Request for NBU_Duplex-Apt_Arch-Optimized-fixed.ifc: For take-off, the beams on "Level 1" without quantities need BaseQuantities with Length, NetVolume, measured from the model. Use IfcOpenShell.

First a look at what the model holds.

```python
import ifcopenshell
import ifcopenshell.util.element
import ifcopenshell.util.unit

model = ifcopenshell.open("NBU_Duplex-Apt_Arch-Optimized-fixed.ifc")
print(model.schema)
for unit_type in ("LENGTHUNIT", "AREAUNIT", "VOLUMEUNIT"):
    print(unit_type, ifcopenshell.util.unit.calculate_unit_scale(model, unit_type))
storey = next(s for s in model.by_type("IfcBuildingStorey") if s.Name == "Level 1")
beams = [e for e in ifcopenshell.util.element.get_decomposition(storey) if e.is_a("IfcBeam")]
for e in sorted(beams, key=lambda e: e.id()):
    print(e.id(), e.is_a(), e.Name, list(ifcopenshell.util.element.get_psets(e, qtos_only=True)), sep=" | ")
```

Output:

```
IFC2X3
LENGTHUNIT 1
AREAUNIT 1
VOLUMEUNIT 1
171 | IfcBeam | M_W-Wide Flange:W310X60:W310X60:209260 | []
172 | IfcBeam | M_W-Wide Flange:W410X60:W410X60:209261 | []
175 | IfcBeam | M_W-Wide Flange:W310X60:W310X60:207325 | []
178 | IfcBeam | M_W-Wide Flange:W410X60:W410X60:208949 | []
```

```python
import ifcopenshell
import ifcopenshell.api.pset
import ifcopenshell.geom
import ifcopenshell.util.element
import ifcopenshell.util.shape
import ifcopenshell.util.unit

model = ifcopenshell.open("NBU_Duplex-Apt_Arch-Optimized-fixed.ifc")
unit_scale = ifcopenshell.util.unit.calculate_unit_scale(model)
volume_scale = ifcopenshell.util.unit.calculate_unit_scale(model, "VOLUMEUNIT")
settings = ifcopenshell.geom.settings()

storey = next(s for s in model.by_type("IfcBuildingStorey") if s.Name == "Level 1")
beams = [e for e in ifcopenshell.util.element.get_decomposition(storey) if e.is_a("IfcBeam")]

for e in sorted(beams, key=lambda e: e.id()):
    if ifcopenshell.util.element.get_psets(e, qtos_only=True, should_inherit=False):
        continue
    # Geometry comes back in metres, in the element's own axes.
    shape = ifcopenshell.geom.create_shape(settings, e)
    values = {
        "Length": ifcopenshell.util.shape.get_max_xyz(shape.geometry) / unit_scale,
        "NetVolume": ifcopenshell.util.shape.get_volume(shape.geometry) / volume_scale,
    }
    qto = ifcopenshell.api.pset.add_qto(model, product=e, name="BaseQuantities")
    ifcopenshell.api.pset.edit_qto(model, qto=qto, properties=values)
    print(e.id(), {k: round(v, 3) for k, v in values.items()})

model.write("NBU_Duplex-Apt_Arch-Optimized-fixed_v2.ifc")
```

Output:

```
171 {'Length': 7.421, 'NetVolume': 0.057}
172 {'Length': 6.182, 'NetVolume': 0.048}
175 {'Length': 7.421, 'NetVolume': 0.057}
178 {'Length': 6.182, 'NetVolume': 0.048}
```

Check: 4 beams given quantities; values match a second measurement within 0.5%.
